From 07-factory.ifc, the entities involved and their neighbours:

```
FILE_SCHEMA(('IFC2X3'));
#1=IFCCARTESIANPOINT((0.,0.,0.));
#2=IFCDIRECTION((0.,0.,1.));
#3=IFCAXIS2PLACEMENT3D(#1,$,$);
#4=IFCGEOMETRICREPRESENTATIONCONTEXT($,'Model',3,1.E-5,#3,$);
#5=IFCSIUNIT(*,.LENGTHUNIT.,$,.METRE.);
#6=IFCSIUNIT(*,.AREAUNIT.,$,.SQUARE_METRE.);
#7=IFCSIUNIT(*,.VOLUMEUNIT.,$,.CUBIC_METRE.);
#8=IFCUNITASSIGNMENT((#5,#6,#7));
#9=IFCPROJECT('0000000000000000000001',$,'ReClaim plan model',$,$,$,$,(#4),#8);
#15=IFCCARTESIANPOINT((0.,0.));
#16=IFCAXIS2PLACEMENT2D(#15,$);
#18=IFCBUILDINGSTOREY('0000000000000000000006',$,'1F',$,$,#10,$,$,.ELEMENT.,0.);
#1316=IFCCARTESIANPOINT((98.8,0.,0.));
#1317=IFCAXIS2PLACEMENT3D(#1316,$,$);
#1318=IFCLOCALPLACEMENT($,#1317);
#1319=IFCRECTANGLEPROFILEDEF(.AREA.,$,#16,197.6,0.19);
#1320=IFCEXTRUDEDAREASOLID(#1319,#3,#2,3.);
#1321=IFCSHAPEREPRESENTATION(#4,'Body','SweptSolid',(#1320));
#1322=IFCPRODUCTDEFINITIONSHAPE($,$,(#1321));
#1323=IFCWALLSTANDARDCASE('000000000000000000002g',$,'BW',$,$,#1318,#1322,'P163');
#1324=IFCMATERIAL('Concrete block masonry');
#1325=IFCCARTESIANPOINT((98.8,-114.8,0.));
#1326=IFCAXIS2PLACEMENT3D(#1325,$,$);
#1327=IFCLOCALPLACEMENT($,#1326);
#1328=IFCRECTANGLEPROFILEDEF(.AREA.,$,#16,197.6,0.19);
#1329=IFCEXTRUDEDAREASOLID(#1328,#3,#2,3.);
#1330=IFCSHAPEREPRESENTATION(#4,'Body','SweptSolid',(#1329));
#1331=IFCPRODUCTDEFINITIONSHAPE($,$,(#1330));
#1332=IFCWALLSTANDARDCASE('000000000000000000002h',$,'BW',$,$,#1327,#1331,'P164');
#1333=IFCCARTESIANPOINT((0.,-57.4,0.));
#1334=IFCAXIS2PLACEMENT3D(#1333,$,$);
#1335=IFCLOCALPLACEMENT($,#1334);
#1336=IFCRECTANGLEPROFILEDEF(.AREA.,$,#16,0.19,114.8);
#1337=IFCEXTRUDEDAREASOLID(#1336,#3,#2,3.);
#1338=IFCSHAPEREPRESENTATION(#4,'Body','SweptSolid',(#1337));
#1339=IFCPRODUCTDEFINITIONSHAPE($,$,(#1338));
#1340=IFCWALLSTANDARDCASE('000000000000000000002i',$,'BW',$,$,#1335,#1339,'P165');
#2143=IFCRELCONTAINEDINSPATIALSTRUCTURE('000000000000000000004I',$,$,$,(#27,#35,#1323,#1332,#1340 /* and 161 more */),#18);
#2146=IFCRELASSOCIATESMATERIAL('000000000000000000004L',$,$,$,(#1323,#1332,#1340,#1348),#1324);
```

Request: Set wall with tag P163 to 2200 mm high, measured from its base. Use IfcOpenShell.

```python
import ifcopenshell
import ifcopenshell.geom
import ifcopenshell.util.shape
import ifcopenshell.util.unit

model = ifcopenshell.open("07-factory.ifc")
unit_scale = ifcopenshell.util.unit.calculate_unit_scale(model)
settings = ifcopenshell.geom.settings()


def volume(element):
    """Net volume in cubic metres, openings subtracted."""
    shape = ifcopenshell.geom.create_shape(settings, element)
    return ifcopenshell.util.shape.get_volume(shape.geometry)


wall = model.by_guid("000000000000000000002g")
before = volume(wall)

body = next(r for r in wall.Representation.Representations if r.RepresentationIdentifier == "Body")
solid = body.Items[0]
old_height = solid.Depth
solid.Depth = 2.2 / unit_scale
after = volume(wall)

print(f"height {old_height:g} -> {solid.Depth:g}, volume {before:.3f} -> {after:.3f} m3")

model.write("07-factory_rev.ifc")
```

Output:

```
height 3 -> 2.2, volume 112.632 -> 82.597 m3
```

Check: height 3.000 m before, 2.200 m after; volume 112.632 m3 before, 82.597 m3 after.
